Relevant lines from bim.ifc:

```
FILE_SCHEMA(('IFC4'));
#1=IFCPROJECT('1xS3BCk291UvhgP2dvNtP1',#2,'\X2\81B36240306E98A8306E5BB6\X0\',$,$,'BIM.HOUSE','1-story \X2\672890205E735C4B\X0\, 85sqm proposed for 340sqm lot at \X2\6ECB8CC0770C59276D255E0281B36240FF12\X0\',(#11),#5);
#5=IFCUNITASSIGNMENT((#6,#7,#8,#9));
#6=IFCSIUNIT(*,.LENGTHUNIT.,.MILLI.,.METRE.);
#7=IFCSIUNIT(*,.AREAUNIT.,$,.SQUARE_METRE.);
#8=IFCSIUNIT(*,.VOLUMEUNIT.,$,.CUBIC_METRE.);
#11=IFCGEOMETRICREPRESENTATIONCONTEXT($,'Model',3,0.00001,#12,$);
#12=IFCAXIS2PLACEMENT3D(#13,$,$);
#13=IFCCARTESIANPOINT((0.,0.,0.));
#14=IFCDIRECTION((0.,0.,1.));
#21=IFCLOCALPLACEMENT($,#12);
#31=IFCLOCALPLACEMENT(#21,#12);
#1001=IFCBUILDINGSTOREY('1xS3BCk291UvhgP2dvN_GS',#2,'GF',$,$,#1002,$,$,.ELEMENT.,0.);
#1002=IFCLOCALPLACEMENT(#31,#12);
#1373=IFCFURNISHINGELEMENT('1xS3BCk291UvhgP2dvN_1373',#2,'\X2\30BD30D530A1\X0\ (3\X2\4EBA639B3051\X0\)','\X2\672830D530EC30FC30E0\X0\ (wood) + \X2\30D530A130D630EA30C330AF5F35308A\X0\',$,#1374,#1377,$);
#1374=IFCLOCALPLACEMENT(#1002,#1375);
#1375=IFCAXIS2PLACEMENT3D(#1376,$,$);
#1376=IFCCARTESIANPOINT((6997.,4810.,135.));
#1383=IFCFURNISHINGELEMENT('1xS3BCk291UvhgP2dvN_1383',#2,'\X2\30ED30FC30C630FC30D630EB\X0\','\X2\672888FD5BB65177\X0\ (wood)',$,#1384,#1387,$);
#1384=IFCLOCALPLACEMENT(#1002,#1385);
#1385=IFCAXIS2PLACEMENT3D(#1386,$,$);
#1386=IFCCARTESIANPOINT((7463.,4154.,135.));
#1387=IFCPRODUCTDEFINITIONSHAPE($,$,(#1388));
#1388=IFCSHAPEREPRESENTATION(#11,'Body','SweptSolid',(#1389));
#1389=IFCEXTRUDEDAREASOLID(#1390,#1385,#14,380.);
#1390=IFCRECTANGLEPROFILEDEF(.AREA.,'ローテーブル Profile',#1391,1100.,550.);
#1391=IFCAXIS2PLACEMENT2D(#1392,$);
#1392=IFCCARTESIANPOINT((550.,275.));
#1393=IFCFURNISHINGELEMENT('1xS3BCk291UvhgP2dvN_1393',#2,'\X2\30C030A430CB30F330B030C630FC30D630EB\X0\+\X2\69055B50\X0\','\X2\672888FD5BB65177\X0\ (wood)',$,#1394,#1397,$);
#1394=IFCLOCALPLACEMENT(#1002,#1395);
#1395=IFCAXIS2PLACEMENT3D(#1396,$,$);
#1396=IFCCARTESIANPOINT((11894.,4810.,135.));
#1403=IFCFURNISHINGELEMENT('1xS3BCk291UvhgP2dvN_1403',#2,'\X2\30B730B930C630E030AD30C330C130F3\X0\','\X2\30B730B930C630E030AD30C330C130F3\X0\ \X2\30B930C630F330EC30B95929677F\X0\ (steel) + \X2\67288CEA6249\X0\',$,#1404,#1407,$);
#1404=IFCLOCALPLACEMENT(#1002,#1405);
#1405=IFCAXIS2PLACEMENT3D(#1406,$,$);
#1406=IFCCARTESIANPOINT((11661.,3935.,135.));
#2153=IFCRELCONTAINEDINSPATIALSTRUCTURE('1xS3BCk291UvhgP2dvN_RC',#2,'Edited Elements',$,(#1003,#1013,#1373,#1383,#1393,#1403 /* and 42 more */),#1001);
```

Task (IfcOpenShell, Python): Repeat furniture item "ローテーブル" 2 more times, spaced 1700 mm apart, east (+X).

```python
import numpy as np
import ifcopenshell
import ifcopenshell.api.geometry
import ifcopenshell.api.root
import ifcopenshell.util.element
import ifcopenshell.util.placement

model = ifcopenshell.open("bim.ifc")


def reuse_history(source, copy):
    """copy_class also copies each property set's owner history, people and application; keep the originals."""
    for rel in copy.IsDefinedBy:
        if rel.is_a("IfcRelDefinesByProperties") and (history := rel.RelatingPropertyDefinition.OwnerHistory):
            rel.RelatingPropertyDefinition.OwnerHistory = source.OwnerHistory
            ifcopenshell.util.element.remove_deep2(model, history)


source = model.by_guid("1xS3BCk291UvhgP2dvN_1383")
base = ifcopenshell.util.placement.get_local_placement(source.ObjectPlacement)
step = np.array([1.0, 0.0, 0.0]) * 1700.0

for i in range(1, 3):
    copy = ifcopenshell.api.root.copy_class(model, product=source)
    copy.Representation = ifcopenshell.util.element.copy_deep(
        model, source.Representation, exclude=["IfcGeometricRepresentationContext", "IfcRepresentationMap"]
    )
    reuse_history(source, copy)
    matrix = base.copy()
    matrix[:3, 3] += i * step
    print("added at", matrix[:3, 3].round(3) + 0.0)
    ifcopenshell.api.geometry.edit_object_placement(model, product=copy, matrix=matrix, is_si=False)

model.write("bim_updated.ifc")
```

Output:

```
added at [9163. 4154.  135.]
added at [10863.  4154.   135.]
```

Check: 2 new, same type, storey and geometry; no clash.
